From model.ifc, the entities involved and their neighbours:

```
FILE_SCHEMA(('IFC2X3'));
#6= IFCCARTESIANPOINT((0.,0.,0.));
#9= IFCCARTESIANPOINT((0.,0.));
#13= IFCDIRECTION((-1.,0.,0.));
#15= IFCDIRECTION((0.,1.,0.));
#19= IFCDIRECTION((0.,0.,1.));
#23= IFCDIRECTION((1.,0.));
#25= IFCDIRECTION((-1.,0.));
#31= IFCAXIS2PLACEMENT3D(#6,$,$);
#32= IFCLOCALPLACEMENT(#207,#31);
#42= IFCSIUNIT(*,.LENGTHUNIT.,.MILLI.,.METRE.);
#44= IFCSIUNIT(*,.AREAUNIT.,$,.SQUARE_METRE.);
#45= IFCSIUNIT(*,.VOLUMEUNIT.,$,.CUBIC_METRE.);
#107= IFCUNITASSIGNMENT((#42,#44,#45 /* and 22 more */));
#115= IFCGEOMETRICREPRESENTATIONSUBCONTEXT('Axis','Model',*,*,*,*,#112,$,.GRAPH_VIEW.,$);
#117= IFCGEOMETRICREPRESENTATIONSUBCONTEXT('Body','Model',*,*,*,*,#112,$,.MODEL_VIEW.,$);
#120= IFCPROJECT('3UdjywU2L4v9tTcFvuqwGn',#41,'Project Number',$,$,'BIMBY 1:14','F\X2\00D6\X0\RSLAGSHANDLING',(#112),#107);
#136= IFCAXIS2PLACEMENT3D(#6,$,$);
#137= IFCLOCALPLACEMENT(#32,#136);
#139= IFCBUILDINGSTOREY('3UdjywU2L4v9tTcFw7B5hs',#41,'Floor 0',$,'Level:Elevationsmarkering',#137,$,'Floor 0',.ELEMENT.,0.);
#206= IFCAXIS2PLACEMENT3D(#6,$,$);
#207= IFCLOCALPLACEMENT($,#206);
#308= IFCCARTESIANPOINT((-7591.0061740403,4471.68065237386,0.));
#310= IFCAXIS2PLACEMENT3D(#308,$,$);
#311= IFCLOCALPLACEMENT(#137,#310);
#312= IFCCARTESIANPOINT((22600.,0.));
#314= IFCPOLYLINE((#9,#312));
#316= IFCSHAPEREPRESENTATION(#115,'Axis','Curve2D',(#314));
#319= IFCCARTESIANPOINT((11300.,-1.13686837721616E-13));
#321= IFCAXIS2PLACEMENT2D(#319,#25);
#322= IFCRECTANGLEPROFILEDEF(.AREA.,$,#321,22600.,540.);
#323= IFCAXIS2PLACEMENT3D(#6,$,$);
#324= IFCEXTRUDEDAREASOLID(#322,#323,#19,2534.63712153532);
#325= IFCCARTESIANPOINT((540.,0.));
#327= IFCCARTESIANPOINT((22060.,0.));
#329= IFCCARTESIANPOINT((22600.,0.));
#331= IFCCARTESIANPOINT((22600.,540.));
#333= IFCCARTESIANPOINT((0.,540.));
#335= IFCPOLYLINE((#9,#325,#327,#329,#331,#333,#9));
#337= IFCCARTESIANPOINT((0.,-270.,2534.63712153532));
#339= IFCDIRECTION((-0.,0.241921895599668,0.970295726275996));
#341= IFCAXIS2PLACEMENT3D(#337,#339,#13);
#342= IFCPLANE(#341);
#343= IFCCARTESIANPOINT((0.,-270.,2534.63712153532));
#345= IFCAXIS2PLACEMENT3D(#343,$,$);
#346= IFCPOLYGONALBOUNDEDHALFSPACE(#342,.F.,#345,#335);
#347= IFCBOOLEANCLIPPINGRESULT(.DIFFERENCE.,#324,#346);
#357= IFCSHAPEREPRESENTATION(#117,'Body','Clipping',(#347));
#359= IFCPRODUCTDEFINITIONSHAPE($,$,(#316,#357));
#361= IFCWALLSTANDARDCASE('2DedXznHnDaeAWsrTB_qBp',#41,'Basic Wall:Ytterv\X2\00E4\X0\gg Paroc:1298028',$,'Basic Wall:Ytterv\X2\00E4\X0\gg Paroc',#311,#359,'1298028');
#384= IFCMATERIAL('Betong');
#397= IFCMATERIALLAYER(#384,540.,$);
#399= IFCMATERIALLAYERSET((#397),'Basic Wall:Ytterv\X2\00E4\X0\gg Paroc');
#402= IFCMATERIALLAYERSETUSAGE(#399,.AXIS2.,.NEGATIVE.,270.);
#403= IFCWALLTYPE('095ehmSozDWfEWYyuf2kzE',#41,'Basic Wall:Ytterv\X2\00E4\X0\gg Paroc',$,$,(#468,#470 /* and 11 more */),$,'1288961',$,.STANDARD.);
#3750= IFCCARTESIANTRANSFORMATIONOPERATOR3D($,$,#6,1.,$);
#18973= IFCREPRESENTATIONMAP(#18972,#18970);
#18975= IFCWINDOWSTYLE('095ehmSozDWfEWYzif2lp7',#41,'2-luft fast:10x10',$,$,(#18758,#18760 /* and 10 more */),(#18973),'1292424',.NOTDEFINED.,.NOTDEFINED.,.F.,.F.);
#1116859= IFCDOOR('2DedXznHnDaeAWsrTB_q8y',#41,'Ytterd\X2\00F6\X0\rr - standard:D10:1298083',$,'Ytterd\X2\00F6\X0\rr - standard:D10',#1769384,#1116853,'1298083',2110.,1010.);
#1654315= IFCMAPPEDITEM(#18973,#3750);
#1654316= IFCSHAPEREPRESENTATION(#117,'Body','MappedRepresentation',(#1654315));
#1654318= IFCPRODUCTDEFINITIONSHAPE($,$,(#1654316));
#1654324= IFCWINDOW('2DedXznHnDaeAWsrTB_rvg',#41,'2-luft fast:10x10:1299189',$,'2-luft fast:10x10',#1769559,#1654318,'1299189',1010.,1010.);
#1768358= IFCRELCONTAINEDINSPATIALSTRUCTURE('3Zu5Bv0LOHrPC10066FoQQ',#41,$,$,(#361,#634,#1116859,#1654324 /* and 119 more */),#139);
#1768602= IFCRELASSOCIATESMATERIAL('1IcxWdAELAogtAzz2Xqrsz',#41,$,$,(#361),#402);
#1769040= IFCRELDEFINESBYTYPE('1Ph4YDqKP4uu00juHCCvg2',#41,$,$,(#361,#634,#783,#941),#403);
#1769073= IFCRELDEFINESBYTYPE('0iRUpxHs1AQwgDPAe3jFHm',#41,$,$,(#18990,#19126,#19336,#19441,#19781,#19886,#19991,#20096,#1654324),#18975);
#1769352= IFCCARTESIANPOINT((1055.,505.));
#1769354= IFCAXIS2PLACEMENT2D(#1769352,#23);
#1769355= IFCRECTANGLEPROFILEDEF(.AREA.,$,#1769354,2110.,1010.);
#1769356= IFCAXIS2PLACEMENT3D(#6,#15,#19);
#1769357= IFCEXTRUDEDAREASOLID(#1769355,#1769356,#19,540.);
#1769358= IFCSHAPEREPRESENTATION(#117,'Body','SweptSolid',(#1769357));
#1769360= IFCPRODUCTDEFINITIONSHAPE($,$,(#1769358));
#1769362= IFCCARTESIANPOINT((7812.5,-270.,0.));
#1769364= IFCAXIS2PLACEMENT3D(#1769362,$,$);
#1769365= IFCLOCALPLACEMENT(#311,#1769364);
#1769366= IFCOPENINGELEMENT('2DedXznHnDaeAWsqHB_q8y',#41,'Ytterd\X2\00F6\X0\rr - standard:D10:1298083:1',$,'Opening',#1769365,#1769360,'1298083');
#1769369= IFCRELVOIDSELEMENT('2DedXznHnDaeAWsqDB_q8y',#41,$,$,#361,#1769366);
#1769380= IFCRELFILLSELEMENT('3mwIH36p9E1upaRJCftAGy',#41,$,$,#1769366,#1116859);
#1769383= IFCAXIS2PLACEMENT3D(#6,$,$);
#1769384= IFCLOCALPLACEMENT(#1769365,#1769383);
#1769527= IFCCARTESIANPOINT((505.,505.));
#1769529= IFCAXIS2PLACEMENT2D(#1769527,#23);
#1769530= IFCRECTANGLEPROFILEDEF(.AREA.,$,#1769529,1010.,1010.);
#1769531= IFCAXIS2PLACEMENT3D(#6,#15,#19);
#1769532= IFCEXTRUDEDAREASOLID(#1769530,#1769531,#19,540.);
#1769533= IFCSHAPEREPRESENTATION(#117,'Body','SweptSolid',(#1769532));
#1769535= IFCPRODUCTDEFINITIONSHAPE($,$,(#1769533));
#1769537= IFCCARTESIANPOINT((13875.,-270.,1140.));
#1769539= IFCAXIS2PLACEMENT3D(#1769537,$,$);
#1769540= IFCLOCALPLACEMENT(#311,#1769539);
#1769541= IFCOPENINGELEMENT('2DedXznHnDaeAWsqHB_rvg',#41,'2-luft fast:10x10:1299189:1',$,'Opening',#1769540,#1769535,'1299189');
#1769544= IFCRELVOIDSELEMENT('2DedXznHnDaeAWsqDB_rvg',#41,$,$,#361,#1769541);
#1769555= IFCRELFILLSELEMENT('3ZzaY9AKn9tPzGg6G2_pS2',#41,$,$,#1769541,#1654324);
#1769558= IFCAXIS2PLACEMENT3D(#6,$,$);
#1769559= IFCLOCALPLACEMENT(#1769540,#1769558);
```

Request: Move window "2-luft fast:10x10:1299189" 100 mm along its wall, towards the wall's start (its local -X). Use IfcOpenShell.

```python
import ifcopenshell
import ifcopenshell.api.geometry
import ifcopenshell.util.placement
import ifcopenshell.util.unit

model = ifcopenshell.open("model.ifc")
unit_scale = ifcopenshell.util.unit.calculate_unit_scale(model)

window = model.by_id(1654324)
opening = window.FillsVoids[0].RelatingOpeningElement
wall = opening.VoidsElements[0].RelatingBuildingElement

wall_matrix = ifcopenshell.util.placement.get_local_placement(wall.ObjectPlacement)
shift = wall_matrix[:3, 0] * -0.1 / unit_scale
before = ifcopenshell.util.placement.get_local_placement(window.ObjectPlacement)[:3, 3].copy()

# The window is placed relative to its opening, so it follows when the opening moves.
matrix = ifcopenshell.util.placement.get_local_placement(opening.ObjectPlacement)
matrix[:3, 3] += shift
ifcopenshell.api.geometry.edit_object_placement(
    model, product=opening, matrix=matrix, is_si=False, should_transform_children=True
)

after = ifcopenshell.util.placement.get_local_placement(window.ObjectPlacement)[:3, 3]
print("window moved by", (after - before).round(3) + 0.0)

model.write("model-out.ifc")
```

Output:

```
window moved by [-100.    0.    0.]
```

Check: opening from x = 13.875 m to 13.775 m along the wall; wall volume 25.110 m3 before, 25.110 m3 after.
